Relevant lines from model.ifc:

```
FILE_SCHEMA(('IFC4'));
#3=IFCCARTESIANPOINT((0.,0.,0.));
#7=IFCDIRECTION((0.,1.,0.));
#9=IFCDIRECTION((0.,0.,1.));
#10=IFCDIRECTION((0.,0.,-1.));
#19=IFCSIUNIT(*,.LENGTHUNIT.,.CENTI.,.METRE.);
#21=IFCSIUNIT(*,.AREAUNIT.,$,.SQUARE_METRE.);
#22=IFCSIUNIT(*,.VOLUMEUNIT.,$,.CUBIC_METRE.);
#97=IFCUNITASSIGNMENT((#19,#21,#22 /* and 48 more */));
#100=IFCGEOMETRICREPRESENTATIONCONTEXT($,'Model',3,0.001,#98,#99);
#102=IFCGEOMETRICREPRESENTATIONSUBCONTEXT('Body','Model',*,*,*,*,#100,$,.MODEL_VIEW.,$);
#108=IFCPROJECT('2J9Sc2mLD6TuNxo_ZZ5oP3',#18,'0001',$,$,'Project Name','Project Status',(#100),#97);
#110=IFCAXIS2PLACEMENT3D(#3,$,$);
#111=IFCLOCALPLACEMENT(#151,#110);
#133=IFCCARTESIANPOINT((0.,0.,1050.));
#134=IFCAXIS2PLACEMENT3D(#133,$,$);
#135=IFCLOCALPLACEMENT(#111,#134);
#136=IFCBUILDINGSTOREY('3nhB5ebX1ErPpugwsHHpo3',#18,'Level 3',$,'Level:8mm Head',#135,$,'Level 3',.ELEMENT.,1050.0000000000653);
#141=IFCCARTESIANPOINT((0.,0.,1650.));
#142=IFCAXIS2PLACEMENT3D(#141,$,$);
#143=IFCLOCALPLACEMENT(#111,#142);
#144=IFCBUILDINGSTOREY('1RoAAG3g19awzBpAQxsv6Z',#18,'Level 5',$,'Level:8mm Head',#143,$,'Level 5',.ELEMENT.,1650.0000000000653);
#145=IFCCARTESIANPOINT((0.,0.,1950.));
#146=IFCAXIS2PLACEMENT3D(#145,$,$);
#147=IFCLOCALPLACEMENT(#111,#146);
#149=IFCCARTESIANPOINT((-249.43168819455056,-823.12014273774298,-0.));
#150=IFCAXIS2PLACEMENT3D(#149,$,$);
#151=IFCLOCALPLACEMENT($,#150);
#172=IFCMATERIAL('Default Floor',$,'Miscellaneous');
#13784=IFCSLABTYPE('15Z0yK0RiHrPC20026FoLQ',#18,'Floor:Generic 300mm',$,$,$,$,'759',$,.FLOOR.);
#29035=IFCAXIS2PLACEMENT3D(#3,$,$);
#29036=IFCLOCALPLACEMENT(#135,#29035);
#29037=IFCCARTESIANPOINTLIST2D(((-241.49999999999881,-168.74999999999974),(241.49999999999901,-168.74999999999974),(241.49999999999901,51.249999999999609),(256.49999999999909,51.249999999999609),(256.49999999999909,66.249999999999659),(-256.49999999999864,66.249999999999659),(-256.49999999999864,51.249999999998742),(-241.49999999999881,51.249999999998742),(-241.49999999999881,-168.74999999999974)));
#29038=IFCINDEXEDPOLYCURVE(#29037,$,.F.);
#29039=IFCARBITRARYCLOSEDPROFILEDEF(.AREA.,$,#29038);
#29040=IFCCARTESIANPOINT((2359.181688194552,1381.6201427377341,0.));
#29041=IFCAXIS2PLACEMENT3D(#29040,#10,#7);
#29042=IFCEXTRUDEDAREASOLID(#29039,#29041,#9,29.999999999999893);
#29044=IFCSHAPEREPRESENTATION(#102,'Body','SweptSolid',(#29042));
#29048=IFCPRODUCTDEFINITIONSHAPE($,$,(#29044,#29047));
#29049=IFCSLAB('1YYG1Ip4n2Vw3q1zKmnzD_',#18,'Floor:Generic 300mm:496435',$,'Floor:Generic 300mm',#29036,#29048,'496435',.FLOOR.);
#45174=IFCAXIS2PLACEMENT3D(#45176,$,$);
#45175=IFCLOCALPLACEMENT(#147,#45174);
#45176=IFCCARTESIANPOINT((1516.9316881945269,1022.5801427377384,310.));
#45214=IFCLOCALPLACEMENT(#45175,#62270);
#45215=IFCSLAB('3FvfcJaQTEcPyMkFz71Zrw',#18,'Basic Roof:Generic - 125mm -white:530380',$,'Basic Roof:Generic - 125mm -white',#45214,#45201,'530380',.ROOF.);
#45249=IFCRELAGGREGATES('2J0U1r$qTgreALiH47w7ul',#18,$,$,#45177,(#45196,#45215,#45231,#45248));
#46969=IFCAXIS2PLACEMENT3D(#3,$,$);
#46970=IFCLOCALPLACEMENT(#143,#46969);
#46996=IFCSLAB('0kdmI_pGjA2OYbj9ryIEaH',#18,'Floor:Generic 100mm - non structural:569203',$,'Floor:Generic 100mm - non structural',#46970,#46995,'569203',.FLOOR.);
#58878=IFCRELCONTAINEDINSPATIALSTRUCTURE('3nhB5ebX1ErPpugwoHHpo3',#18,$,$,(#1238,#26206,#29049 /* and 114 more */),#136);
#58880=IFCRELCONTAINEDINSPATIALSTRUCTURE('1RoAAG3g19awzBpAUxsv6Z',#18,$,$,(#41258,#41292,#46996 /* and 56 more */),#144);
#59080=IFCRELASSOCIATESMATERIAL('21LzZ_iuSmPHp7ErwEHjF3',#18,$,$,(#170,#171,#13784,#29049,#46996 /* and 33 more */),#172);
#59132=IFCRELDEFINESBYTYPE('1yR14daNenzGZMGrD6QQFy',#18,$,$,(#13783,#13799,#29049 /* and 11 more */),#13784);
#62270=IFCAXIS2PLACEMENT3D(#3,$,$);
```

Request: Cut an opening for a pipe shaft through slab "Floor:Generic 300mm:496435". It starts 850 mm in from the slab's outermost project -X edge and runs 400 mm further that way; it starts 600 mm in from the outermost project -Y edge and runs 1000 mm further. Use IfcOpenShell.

```python
import numpy as np
import ifcopenshell
import ifcopenshell.api.feature
import ifcopenshell.api.geometry
import ifcopenshell.api.root
import ifcopenshell.geom
import ifcopenshell.util.placement
import ifcopenshell.util.representation
import ifcopenshell.util.shape
import ifcopenshell.util.unit

model = ifcopenshell.open("model.ifc")
unit_scale = ifcopenshell.util.unit.calculate_unit_scale(model)
settings = ifcopenshell.geom.settings()


def volume(element):
    """Net volume in cubic metres, openings subtracted."""
    shape = ifcopenshell.geom.create_shape(settings, element)
    return ifcopenshell.util.shape.get_volume(shape.geometry)


slab = model.by_guid("1YYG1Ip4n2Vw3q1zKmnzD_")
before = volume(slab)

# Extent in the slab's own axes, in metres. The edges named are its -X and -Y sides.
slab_shape = ifcopenshell.geom.create_shape(settings, slab)
vertices = ifcopenshell.util.shape.get_vertices(slab_shape.geometry)
x_min, y_min, bottom = vertices.min(axis=0)
top = vertices[:, 2].max()

opening = ifcopenshell.api.root.create_entity(model, ifc_class="IfcOpeningElement", name="Pipe shaft opening", predefined_type="OPENING")
context = ifcopenshell.util.representation.get_context(model, "Model", "Body", "MODEL_VIEW")
width, depth = 0.4, 1
outline = [(0.0, 0.0), (width, 0.0), (width, depth), (0.0, depth), (0.0, 0.0)]
# Overshoot both faces by 50 mm so the cut is clean.
shape = ifcopenshell.api.geometry.add_slab_representation(
    model, context=context, depth=top - bottom + 0.1, polyline=outline
)
ifcopenshell.api.geometry.assign_representation(model, product=opening, representation=shape)

matrix = ifcopenshell.util.placement.get_local_placement(slab.ObjectPlacement)
matrix[:, 3] = matrix @ np.append(np.array([x_min + 0.85, y_min + 0.6, bottom - 0.05]) / unit_scale, 1.0)
ifcopenshell.api.geometry.edit_object_placement(model, product=opening, matrix=matrix, is_si=False)
ifcopenshell.api.feature.add_feature(model, feature=opening, element=slab)

after = volume(slab)

print(f"slab volume {before:.3f} -> {after:.3f} m3")

model.write("model_rev.ifc")
```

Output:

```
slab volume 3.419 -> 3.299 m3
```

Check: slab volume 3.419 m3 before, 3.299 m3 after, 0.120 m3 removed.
